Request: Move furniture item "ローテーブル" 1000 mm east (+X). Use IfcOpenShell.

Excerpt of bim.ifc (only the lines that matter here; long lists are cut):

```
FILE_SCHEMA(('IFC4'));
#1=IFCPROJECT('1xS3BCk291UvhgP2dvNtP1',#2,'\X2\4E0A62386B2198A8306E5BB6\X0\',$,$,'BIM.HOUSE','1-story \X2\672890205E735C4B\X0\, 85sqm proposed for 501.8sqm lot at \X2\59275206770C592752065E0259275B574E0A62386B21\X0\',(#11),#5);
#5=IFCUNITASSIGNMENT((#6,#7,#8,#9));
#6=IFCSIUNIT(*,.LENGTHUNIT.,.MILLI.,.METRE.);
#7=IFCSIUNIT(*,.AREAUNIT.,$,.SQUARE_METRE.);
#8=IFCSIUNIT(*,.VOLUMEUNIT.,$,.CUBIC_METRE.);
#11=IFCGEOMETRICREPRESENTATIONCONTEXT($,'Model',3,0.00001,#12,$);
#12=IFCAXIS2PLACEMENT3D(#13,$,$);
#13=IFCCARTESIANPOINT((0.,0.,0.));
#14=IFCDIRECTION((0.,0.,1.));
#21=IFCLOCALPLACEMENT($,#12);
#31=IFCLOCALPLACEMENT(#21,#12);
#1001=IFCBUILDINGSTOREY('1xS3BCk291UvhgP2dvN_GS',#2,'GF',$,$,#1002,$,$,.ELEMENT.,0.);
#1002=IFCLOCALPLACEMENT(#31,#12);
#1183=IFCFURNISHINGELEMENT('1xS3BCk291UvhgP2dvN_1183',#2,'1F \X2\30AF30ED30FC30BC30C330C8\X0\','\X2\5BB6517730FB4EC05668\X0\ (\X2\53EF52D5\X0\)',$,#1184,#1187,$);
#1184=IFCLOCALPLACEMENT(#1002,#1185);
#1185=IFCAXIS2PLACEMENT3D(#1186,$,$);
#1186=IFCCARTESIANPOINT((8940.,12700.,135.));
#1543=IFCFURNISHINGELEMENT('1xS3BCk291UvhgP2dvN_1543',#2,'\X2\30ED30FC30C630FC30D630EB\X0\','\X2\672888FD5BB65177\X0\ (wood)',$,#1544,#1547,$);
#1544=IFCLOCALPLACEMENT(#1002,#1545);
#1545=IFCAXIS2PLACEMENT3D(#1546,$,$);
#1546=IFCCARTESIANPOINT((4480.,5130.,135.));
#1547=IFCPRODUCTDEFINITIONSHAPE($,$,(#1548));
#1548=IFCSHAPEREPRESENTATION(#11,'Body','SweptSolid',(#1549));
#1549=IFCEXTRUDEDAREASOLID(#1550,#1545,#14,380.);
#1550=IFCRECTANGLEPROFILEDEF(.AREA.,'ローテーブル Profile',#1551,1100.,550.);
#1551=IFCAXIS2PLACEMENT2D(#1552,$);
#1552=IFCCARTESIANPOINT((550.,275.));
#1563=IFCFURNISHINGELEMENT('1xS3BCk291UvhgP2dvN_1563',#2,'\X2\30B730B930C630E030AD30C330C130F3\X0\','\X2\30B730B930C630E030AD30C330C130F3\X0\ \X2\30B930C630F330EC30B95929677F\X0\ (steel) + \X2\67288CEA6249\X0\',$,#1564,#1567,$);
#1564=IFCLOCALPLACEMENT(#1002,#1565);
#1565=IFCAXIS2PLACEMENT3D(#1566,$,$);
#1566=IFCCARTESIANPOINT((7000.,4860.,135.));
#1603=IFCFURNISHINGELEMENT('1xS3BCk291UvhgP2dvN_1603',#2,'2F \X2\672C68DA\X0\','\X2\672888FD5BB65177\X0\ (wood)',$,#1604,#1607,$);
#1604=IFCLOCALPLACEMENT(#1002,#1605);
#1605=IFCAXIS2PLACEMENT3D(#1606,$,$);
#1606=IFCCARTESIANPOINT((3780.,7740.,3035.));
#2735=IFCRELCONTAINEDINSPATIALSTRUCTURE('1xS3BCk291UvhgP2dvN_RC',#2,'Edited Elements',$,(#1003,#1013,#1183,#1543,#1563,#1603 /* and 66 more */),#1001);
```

```python
import ifcopenshell
import ifcopenshell.api.geometry
import ifcopenshell.util.placement
import ifcopenshell.util.unit

model = ifcopenshell.open("bim.ifc")
unit_scale = ifcopenshell.util.unit.calculate_unit_scale(model)

item = model.by_guid("1xS3BCk291UvhgP2dvN_1543")
matrix = ifcopenshell.util.placement.get_local_placement(item.ObjectPlacement)
matrix[0, 3] += 1 / unit_scale
ifcopenshell.api.geometry.edit_object_placement(model, product=item, matrix=matrix, is_si=False)

print(ifcopenshell.util.placement.get_local_placement(item.ObjectPlacement).round(3) + 0.0)

model.write("bim_v2.ifc")
```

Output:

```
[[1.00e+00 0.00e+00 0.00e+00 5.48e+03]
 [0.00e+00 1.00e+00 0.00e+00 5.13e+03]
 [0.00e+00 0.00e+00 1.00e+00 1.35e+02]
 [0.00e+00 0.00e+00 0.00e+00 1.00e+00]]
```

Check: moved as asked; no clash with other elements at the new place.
